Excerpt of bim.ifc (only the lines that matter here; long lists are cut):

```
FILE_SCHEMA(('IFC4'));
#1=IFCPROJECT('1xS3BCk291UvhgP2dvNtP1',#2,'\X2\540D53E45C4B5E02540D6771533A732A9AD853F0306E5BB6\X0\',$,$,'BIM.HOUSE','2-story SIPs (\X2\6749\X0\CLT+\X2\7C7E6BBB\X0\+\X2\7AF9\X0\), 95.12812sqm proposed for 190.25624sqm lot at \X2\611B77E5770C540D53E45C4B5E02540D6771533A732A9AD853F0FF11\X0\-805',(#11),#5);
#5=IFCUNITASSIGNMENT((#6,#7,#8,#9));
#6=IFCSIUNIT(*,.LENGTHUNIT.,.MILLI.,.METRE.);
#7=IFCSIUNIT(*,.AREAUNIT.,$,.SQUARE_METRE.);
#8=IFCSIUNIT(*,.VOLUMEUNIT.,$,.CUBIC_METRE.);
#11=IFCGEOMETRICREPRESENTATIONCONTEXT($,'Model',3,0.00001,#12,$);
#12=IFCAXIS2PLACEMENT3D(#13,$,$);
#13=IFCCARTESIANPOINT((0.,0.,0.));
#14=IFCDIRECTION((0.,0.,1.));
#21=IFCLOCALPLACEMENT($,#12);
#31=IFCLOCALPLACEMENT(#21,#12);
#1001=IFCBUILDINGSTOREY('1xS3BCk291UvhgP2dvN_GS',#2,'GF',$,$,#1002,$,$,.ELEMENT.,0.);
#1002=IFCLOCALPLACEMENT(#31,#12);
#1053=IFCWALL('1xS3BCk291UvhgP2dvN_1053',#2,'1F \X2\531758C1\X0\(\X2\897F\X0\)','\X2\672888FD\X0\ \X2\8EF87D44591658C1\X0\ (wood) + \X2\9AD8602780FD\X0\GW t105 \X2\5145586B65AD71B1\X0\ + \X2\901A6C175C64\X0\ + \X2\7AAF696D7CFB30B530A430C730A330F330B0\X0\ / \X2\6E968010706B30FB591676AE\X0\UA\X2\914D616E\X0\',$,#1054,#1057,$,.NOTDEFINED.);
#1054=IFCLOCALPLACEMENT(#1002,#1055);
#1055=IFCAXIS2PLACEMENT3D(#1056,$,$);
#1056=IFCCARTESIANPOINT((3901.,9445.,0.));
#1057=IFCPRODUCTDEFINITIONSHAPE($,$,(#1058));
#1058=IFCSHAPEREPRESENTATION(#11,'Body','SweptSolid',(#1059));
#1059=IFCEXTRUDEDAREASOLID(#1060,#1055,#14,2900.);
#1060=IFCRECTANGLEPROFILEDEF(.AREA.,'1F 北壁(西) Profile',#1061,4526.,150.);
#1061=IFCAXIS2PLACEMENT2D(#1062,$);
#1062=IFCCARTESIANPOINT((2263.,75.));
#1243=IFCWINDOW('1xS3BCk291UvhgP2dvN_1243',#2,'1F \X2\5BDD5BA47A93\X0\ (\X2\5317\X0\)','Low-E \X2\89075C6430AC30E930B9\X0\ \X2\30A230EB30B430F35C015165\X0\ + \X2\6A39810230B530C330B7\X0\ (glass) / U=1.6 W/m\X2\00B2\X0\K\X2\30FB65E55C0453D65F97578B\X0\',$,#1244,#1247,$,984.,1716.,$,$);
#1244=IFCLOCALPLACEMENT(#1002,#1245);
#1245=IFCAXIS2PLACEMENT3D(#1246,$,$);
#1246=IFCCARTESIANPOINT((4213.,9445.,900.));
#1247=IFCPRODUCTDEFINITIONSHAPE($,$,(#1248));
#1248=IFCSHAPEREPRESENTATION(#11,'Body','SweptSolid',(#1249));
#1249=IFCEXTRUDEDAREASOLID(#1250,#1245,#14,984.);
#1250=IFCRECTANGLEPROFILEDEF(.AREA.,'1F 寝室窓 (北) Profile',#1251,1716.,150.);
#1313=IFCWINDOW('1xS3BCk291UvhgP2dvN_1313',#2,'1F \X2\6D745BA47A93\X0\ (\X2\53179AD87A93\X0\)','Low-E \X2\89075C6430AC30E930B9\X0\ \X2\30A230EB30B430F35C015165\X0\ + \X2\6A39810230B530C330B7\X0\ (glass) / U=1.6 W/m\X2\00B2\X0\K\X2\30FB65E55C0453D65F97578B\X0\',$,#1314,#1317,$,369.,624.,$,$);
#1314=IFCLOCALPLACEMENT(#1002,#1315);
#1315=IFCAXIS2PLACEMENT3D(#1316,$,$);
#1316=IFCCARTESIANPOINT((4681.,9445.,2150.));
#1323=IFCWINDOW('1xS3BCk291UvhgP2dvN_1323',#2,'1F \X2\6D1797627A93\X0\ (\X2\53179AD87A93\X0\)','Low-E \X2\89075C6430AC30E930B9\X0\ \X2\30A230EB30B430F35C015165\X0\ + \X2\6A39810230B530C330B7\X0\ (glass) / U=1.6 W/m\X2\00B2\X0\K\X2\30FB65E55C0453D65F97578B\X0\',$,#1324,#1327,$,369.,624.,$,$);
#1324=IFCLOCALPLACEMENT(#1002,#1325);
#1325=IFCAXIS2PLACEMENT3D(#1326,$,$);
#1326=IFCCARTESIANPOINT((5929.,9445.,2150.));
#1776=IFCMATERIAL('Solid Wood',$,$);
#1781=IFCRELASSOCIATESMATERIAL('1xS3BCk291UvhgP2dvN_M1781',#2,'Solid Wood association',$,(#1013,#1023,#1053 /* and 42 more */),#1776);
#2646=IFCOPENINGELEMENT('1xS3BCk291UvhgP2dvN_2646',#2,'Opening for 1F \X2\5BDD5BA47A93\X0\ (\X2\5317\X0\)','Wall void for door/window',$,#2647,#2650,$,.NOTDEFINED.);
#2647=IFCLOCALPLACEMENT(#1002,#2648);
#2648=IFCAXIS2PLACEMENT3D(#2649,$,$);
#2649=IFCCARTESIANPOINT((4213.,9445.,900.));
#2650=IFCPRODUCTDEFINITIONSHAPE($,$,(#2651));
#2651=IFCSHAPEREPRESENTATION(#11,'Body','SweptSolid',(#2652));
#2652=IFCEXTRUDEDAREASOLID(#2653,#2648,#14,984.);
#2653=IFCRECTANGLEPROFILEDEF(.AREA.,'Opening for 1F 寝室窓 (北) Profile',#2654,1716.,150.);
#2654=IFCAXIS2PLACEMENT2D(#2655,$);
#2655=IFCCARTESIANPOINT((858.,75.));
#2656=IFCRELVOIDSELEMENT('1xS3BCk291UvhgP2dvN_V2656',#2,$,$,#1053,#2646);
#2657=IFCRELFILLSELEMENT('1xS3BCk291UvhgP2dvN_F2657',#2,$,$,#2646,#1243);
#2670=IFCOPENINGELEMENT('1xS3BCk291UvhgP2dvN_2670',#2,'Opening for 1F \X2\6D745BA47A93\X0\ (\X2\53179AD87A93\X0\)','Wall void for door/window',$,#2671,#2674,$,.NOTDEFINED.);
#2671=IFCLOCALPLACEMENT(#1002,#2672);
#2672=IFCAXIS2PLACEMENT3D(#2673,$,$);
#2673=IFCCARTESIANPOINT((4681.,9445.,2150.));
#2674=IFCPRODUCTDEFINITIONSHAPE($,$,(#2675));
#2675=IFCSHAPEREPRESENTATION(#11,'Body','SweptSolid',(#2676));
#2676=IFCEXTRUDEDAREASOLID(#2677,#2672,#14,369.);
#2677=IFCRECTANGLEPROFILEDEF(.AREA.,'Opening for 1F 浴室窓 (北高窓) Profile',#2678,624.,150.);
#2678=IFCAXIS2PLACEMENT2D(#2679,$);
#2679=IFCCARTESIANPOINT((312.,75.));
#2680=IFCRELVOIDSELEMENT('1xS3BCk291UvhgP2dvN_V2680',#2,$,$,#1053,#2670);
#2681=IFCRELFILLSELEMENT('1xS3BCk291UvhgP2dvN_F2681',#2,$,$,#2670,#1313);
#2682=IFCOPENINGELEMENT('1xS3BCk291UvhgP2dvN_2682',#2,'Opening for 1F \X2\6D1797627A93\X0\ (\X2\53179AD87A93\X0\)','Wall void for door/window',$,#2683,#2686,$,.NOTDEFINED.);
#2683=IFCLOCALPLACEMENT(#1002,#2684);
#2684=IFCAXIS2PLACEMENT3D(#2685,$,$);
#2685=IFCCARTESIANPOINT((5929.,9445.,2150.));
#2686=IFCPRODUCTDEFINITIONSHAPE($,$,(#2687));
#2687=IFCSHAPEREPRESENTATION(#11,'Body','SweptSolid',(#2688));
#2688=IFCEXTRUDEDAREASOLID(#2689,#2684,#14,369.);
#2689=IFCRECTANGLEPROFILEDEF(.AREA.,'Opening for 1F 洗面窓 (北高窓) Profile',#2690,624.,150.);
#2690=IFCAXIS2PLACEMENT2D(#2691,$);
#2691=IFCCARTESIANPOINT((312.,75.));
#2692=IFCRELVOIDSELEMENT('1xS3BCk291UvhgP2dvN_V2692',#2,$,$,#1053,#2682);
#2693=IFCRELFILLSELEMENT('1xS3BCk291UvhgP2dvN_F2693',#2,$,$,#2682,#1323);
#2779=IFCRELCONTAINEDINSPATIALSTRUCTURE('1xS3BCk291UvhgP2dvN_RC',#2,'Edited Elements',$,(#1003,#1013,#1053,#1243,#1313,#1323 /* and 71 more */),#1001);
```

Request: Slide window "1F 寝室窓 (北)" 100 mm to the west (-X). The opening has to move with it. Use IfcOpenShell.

```python
import ifcopenshell
import ifcopenshell.api.geometry
import ifcopenshell.util.placement

model = ifcopenshell.open("bim.ifc")

window = model.by_id(1243)
opening = window.FillsVoids[0].RelatingOpeningElement
wall = opening.VoidsElements[0].RelatingBuildingElement

wall_matrix = ifcopenshell.util.placement.get_local_placement(wall.ObjectPlacement)
shift = wall_matrix[:3, 0] * -100.0
before = ifcopenshell.util.placement.get_local_placement(window.ObjectPlacement)[:3, 3].copy()

# The window is not placed relative to its opening, so move both.
for product in (opening, window):
    matrix = ifcopenshell.util.placement.get_local_placement(product.ObjectPlacement)
    matrix[:3, 3] += shift
    ifcopenshell.api.geometry.edit_object_placement(model, product=product, matrix=matrix, is_si=False)

after = ifcopenshell.util.placement.get_local_placement(window.ObjectPlacement)[:3, 3]
print("window moved by", (after - before).round(3) + 0.0)

model.write("bim_updated.ifc")
```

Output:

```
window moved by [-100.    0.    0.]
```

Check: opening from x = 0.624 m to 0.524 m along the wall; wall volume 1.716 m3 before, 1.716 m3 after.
